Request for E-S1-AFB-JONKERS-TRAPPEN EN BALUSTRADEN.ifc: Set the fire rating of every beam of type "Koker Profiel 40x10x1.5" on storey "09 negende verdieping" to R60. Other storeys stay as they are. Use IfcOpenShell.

First a look at what the model holds.

```python
import ifcopenshell
import ifcopenshell.util.element

model = ifcopenshell.open("E-S1-AFB-JONKERS-TRAPPEN EN BALUSTRADEN.ifc")
print(model.schema)
storey = next(s for s in model.by_type("IfcBuildingStorey") if s.Name == "09 negende verdieping")
beams = [e for e in ifcopenshell.util.element.get_decomposition(storey) if e.is_a("IfcBeam")]
seen = {}
for e in beams:
    element_type = ifcopenshell.util.element.get_type(e)
    key = (element_type.Name if element_type != e and element_type else None, ifcopenshell.util.element.get_pset(e, "Pset_BeamCommon", "FireRating"))
    seen[key] = seen.get(key, 0) + 1
for (name, value), count in sorted(seen.items(), key=str):
    print(count, "x", name, "|", value)
```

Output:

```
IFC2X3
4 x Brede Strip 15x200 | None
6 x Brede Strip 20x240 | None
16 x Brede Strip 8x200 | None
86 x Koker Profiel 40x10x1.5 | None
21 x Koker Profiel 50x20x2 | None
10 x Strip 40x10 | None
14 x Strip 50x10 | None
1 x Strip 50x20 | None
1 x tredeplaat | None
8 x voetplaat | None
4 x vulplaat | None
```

```python
import ifcopenshell
import ifcopenshell.api.pset
import ifcopenshell.util.element

model = ifcopenshell.open("E-S1-AFB-JONKERS-TRAPPEN EN BALUSTRADEN.ifc")

storey = next(s for s in model.by_type("IfcBuildingStorey") if s.Name == "09 negende verdieping")
beams = [e for e in ifcopenshell.util.element.get_decomposition(storey) if e.is_a("IfcBeam")]

count = 0
for e in beams:
    element_type = ifcopenshell.util.element.get_type(e)
    if element_type in (None, e) or element_type.Name != "Koker Profiel 40x10x1.5":
        continue
    # add_pset returns the element's existing set when there is one.
    pset = ifcopenshell.api.pset.add_pset(model, product=e, name="Pset_BeamCommon")
    ifcopenshell.api.pset.edit_pset(model, pset=pset, properties={"FireRating": "R60"})
    count += 1

print(count, "beams updated")

model.write("E-S1-AFB-JONKERS-TRAPPEN EN BALUSTRADEN-out.ifc")
```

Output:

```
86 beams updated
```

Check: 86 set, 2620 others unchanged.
